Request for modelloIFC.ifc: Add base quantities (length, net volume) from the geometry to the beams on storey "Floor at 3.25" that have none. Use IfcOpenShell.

First a look at what the model holds.

```python
import ifcopenshell
import ifcopenshell.util.element
import ifcopenshell.util.unit

model = ifcopenshell.open("modelloIFC.ifc")
print(model.schema)
for unit_type in ("LENGTHUNIT", "AREAUNIT", "VOLUMEUNIT"):
    print(unit_type, ifcopenshell.util.unit.calculate_unit_scale(model, unit_type))
storey = next(s for s in model.by_type("IfcBuildingStorey") if s.Name == "Floor at 3.25")
beams = [e for e in ifcopenshell.util.element.get_decomposition(storey) if e.is_a("IfcBeam")]
for e in sorted(beams, key=lambda e: e.id()):
    print(e.id(), e.is_a(), e.Name, list(ifcopenshell.util.element.get_psets(e, qtos_only=True)), sep=" | ")
```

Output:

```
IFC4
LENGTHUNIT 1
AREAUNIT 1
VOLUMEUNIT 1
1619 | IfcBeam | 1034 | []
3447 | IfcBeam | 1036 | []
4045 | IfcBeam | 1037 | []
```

```python
import ifcopenshell
import ifcopenshell.api.pset
import ifcopenshell.geom
import ifcopenshell.util.element
import ifcopenshell.util.shape
import ifcopenshell.util.unit

model = ifcopenshell.open("modelloIFC.ifc")
unit_scale = ifcopenshell.util.unit.calculate_unit_scale(model)
volume_scale = ifcopenshell.util.unit.calculate_unit_scale(model, "VOLUMEUNIT")
settings = ifcopenshell.geom.settings()

storey = next(s for s in model.by_type("IfcBuildingStorey") if s.Name == "Floor at 3.25")
beams = [e for e in ifcopenshell.util.element.get_decomposition(storey) if e.is_a("IfcBeam")]

for e in sorted(beams, key=lambda e: e.id()):
    if ifcopenshell.util.element.get_psets(e, qtos_only=True, should_inherit=False):
        continue
    # Geometry comes back in metres, in the element's own axes.
    shape = ifcopenshell.geom.create_shape(settings, e)
    values = {
        "Length": ifcopenshell.util.shape.get_max_xyz(shape.geometry) / unit_scale,
        "NetVolume": ifcopenshell.util.shape.get_volume(shape.geometry) / volume_scale,
    }
    qto = ifcopenshell.api.pset.add_qto(model, product=e, name="Qto_BeamBaseQuantities")
    ifcopenshell.api.pset.edit_qto(model, qto=qto, properties=values)
    print(e.id(), {k: round(v, 3) for k, v in values.items()})

model.write("modelloIFC_updated.ifc")
```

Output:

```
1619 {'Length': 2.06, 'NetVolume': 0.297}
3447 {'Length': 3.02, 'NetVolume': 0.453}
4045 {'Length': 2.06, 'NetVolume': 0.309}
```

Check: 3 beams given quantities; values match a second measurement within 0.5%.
